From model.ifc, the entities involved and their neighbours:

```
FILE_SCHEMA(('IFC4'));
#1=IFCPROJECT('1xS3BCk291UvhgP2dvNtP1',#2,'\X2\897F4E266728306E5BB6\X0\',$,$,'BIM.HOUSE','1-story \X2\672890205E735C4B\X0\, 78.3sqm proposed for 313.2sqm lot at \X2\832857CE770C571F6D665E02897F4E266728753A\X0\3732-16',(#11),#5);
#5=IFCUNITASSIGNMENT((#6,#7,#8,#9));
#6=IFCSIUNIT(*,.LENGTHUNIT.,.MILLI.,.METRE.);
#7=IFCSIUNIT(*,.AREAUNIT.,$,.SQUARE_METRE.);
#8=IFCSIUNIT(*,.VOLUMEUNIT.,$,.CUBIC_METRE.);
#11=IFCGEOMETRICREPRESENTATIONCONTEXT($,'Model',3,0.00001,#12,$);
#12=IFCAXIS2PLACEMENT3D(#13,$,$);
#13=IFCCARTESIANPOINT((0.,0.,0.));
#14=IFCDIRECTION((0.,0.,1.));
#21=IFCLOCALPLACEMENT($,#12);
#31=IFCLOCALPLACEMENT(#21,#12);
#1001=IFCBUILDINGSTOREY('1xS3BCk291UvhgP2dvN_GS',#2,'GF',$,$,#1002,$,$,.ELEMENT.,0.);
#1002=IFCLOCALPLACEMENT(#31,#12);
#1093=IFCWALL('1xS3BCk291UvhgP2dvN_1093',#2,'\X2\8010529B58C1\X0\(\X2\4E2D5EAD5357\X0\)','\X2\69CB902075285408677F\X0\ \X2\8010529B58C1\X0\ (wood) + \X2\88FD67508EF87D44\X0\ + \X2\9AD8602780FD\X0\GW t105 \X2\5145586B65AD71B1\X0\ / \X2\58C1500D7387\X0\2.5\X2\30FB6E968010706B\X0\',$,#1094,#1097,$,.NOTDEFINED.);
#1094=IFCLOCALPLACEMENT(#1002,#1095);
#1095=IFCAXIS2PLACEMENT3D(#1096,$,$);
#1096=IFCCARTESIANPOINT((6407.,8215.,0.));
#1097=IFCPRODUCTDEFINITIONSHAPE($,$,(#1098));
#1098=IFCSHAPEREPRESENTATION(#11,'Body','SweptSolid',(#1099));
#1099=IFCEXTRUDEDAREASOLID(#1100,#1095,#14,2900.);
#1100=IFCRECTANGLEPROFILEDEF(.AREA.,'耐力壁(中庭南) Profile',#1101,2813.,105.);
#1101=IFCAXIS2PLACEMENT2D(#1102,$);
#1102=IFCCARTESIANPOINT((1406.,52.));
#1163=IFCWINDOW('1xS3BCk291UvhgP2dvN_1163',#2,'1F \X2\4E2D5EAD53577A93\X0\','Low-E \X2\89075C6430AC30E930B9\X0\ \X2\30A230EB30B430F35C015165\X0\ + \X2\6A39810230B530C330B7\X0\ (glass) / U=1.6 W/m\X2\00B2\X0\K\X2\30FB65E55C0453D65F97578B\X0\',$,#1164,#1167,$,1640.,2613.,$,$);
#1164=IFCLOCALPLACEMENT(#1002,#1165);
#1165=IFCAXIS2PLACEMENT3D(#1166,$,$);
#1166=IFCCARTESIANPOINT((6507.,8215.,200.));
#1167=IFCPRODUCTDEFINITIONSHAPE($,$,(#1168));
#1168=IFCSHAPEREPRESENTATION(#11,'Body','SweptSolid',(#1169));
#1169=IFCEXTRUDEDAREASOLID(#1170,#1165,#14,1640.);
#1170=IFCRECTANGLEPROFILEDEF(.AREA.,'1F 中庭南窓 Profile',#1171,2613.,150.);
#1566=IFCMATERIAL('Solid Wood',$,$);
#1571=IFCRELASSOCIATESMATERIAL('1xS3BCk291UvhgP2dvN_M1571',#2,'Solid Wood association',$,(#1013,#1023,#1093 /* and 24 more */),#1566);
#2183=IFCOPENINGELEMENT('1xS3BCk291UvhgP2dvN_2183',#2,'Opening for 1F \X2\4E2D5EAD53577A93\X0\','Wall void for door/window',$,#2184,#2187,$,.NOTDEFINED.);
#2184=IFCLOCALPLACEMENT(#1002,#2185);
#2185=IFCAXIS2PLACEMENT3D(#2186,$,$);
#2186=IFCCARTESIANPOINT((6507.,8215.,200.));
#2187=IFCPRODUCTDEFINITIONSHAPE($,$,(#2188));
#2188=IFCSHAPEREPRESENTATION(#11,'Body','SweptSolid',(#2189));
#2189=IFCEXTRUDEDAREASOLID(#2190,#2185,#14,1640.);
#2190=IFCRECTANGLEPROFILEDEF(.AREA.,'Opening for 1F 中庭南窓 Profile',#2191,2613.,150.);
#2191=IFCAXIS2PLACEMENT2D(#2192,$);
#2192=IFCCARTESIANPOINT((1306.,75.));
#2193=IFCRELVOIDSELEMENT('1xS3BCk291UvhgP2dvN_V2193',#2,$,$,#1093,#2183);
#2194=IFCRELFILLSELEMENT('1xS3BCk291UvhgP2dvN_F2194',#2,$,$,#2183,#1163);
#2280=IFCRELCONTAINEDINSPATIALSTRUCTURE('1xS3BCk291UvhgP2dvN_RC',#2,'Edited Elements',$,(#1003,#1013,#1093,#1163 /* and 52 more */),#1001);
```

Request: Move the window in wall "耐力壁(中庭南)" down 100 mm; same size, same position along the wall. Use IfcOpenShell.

```python
import numpy as np
import ifcopenshell
import ifcopenshell.api.geometry
import ifcopenshell.util.placement
import ifcopenshell.util.unit

model = ifcopenshell.open("model.ifc")
unit_scale = ifcopenshell.util.unit.calculate_unit_scale(model)

window = model.by_id(1163)
opening = window.FillsVoids[0].RelatingOpeningElement
dz = -0.1 / unit_scale

shift = np.array([0.0, 0.0, dz])
# The window is not placed relative to its opening, so move both.
for product in (opening, window):
    matrix = ifcopenshell.util.placement.get_local_placement(product.ObjectPlacement)
    matrix[:3, 3] += shift
    ifcopenshell.api.geometry.edit_object_placement(model, product=product, matrix=matrix, is_si=False)

print(f"moved by {dz * unit_scale:+.3f} m")

model.write("model_edited.ifc")
```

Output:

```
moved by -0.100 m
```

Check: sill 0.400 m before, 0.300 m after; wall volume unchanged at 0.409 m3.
